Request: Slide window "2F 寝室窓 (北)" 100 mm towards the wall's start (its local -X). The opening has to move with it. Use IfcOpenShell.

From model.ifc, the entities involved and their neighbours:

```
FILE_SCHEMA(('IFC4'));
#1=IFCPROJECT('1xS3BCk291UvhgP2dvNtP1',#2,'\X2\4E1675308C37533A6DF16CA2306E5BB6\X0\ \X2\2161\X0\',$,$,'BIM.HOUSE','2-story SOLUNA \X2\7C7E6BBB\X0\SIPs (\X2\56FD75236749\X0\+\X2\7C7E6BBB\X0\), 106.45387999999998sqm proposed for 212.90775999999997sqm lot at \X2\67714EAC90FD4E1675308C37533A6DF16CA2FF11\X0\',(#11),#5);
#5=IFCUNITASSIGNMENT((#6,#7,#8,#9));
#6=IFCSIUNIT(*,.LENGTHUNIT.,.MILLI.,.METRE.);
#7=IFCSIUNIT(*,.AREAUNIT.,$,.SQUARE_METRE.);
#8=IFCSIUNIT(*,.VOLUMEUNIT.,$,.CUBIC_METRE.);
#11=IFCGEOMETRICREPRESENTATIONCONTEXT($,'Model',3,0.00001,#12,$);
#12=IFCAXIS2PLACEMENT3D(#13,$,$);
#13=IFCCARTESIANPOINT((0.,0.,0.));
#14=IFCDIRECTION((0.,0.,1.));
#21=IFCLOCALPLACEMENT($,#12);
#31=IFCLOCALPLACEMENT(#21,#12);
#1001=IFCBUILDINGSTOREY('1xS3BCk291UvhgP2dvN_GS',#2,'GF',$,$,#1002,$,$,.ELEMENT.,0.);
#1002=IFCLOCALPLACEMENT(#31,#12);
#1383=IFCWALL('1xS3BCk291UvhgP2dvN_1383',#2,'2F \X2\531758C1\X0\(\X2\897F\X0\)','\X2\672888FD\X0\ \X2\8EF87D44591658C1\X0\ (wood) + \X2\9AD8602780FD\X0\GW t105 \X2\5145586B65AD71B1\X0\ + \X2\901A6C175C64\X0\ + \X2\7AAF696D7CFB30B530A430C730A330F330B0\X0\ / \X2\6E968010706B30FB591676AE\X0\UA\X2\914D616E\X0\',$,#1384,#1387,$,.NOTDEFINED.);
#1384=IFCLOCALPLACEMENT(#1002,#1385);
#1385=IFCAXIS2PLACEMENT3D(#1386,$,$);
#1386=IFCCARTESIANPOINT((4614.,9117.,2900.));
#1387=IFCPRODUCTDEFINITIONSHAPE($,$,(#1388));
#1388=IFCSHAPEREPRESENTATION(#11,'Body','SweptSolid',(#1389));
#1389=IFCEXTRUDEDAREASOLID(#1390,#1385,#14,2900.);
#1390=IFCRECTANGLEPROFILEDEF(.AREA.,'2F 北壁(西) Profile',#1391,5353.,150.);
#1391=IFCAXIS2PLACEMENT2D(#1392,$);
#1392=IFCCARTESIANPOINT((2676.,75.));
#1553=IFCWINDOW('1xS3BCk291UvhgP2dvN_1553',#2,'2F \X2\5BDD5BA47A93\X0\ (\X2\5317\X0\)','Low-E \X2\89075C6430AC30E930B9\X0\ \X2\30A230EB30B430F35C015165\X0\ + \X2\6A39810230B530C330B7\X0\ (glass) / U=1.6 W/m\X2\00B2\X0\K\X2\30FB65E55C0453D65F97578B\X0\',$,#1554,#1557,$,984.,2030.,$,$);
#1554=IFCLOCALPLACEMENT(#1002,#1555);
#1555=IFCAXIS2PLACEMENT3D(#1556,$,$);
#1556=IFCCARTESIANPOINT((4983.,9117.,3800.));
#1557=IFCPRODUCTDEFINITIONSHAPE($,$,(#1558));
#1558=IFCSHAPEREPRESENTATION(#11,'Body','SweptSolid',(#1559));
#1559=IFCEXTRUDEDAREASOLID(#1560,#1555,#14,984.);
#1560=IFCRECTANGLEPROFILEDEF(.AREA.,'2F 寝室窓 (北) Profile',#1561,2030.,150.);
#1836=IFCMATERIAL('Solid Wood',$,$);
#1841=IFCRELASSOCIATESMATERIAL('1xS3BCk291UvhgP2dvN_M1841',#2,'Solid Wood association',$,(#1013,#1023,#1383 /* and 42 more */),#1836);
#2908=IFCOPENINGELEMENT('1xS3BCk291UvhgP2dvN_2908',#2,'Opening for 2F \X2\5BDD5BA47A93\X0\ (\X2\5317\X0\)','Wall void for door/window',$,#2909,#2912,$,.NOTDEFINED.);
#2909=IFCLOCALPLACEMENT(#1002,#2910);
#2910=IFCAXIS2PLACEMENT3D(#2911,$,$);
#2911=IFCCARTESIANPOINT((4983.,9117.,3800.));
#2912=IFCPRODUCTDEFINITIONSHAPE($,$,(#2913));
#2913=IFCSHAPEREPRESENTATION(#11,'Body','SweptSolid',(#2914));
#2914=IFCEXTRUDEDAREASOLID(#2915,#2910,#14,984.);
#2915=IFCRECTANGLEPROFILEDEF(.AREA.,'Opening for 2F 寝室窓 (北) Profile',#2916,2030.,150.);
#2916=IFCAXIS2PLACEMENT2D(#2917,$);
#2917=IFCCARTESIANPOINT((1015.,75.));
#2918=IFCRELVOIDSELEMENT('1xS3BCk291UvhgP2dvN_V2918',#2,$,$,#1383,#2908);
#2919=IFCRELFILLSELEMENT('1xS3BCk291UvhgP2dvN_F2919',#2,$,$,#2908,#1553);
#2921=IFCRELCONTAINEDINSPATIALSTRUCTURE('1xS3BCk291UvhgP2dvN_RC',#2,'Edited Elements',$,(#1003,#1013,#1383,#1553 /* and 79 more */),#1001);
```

```python
import ifcopenshell
import ifcopenshell.api.geometry
import ifcopenshell.util.placement

model = ifcopenshell.open("model.ifc")

window = model.by_guid("1xS3BCk291UvhgP2dvN_1553")
opening = window.FillsVoids[0].RelatingOpeningElement
wall = opening.VoidsElements[0].RelatingBuildingElement

wall_matrix = ifcopenshell.util.placement.get_local_placement(wall.ObjectPlacement)
shift = wall_matrix[:3, 0] * -100.0
before = ifcopenshell.util.placement.get_local_placement(window.ObjectPlacement)[:3, 3].copy()

# The window is not placed relative to its opening, so move both.
for product in (opening, window):
    matrix = ifcopenshell.util.placement.get_local_placement(product.ObjectPlacement)
    matrix[:3, 3] += shift
    ifcopenshell.api.geometry.edit_object_placement(model, product=product, matrix=matrix, is_si=False)

after = ifcopenshell.util.placement.get_local_placement(window.ObjectPlacement)[:3, 3]
print("window moved by", (after - before).round(3) + 0.0)

model.write("model-out.ifc")
```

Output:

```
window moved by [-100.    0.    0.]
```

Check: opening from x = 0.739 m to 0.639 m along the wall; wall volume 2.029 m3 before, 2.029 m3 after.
